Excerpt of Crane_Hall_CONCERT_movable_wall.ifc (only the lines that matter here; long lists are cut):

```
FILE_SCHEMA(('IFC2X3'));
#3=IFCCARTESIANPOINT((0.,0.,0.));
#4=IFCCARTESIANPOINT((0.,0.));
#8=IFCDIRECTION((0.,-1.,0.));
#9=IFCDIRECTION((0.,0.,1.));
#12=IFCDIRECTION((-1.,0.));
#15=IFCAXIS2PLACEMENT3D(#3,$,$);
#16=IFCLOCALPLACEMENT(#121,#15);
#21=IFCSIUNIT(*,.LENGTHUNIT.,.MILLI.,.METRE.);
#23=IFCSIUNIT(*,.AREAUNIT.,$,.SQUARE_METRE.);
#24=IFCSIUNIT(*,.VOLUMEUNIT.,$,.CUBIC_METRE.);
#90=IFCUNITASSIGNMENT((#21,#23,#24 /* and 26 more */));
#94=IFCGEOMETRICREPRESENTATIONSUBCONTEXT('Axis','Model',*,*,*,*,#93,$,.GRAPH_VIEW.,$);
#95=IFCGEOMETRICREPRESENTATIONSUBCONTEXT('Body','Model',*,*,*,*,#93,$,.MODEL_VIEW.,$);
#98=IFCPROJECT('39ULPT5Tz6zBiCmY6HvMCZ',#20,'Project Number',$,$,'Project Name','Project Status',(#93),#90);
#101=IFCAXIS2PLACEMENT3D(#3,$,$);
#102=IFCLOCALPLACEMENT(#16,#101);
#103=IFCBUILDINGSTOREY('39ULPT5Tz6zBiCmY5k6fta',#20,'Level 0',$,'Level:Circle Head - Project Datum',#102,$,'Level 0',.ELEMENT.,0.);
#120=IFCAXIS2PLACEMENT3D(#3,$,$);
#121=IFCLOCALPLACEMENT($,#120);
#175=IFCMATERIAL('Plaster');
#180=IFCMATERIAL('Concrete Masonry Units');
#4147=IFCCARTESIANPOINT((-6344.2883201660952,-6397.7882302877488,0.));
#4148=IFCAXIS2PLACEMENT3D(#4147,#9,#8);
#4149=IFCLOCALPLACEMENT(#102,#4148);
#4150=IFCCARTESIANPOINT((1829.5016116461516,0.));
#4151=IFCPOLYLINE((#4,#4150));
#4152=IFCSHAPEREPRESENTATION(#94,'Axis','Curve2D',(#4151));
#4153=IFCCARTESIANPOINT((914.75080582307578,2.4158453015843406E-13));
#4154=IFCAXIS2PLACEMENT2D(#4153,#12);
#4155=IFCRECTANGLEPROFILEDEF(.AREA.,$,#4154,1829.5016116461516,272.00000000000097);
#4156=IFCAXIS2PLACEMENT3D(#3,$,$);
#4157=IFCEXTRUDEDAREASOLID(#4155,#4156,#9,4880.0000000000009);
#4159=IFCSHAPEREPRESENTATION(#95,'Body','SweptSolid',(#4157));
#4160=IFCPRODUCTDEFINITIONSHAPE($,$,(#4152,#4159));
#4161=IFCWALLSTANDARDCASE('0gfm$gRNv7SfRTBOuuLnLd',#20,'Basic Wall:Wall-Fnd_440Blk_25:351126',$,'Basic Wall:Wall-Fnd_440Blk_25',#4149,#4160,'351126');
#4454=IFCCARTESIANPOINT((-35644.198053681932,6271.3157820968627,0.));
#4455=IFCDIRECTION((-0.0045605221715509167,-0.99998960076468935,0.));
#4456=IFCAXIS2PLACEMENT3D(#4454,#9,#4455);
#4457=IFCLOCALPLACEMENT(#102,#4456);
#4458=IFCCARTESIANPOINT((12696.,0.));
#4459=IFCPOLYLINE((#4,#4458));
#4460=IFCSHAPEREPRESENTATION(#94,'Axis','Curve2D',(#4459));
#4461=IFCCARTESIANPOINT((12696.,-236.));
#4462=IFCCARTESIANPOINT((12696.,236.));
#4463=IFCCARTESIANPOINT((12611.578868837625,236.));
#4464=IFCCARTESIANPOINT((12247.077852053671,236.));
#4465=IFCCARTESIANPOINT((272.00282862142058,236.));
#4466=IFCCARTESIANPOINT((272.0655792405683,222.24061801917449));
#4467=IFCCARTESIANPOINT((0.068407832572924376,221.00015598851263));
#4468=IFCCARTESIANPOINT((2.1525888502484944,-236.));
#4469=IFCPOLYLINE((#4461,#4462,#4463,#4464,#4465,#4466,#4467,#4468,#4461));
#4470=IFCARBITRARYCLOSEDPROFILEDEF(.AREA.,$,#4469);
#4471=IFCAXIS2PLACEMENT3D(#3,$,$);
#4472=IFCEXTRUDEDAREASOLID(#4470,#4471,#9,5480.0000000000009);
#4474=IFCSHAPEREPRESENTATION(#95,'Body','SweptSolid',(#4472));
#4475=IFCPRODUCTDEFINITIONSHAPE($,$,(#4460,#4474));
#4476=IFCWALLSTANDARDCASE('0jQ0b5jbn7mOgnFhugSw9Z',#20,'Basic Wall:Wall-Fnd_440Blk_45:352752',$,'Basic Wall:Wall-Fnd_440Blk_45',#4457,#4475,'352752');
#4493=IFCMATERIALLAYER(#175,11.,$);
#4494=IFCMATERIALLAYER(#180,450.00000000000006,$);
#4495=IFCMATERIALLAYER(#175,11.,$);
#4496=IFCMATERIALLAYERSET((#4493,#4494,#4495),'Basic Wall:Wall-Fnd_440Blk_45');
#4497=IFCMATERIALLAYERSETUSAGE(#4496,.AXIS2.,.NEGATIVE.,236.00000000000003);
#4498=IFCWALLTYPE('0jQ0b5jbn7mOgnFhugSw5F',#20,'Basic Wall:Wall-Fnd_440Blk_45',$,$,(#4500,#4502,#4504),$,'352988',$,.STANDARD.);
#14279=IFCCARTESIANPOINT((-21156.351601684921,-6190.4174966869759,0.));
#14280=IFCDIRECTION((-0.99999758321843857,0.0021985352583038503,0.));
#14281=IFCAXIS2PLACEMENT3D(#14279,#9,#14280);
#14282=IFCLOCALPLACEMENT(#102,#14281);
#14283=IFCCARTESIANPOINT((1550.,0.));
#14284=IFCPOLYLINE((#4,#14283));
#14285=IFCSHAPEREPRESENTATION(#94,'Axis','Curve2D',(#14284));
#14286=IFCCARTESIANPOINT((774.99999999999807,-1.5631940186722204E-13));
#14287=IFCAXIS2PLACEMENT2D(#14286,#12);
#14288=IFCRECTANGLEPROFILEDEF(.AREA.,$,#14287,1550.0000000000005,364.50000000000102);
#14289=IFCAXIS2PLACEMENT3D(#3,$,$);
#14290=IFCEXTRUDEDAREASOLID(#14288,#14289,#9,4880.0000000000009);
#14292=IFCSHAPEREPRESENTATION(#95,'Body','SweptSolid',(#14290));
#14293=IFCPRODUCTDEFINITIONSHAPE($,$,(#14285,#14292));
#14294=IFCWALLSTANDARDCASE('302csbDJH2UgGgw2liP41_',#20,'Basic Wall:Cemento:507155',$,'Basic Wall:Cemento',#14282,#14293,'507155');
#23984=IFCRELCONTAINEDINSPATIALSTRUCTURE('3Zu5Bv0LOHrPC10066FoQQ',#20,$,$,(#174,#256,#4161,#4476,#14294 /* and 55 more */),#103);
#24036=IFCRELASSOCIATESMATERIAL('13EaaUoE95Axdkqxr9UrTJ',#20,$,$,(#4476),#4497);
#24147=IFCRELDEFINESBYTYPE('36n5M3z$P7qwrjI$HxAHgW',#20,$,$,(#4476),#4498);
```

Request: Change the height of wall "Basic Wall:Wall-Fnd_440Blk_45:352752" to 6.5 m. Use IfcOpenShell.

```python
import ifcopenshell
import ifcopenshell.geom
import ifcopenshell.util.representation
import ifcopenshell.util.shape
import ifcopenshell.util.unit

model = ifcopenshell.open("Crane_Hall_CONCERT_movable_wall.ifc")
unit_scale = ifcopenshell.util.unit.calculate_unit_scale(model)
settings = ifcopenshell.geom.settings()


def volume(element):
    """Net volume in cubic metres, openings subtracted."""
    shape = ifcopenshell.geom.create_shape(settings, element)
    return ifcopenshell.util.shape.get_volume(shape.geometry)


wall = model.by_guid("0jQ0b5jbn7mOgnFhugSw9Z")
before = volume(wall)

body = ifcopenshell.util.representation.get_representation(wall, "Model", "Body")
solid = body.Items[0]
old_height = solid.Depth
solid.Depth = 6.5 / unit_scale
after = volume(wall)

print(f"height {old_height:g} -> {solid.Depth:g}, volume {before:.3f} -> {after:.3f} m3")

model.write("Crane_Hall_CONCERT_movable_wall_updated.ifc")
```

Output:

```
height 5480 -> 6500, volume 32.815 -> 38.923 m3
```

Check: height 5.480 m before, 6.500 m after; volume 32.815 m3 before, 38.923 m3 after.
